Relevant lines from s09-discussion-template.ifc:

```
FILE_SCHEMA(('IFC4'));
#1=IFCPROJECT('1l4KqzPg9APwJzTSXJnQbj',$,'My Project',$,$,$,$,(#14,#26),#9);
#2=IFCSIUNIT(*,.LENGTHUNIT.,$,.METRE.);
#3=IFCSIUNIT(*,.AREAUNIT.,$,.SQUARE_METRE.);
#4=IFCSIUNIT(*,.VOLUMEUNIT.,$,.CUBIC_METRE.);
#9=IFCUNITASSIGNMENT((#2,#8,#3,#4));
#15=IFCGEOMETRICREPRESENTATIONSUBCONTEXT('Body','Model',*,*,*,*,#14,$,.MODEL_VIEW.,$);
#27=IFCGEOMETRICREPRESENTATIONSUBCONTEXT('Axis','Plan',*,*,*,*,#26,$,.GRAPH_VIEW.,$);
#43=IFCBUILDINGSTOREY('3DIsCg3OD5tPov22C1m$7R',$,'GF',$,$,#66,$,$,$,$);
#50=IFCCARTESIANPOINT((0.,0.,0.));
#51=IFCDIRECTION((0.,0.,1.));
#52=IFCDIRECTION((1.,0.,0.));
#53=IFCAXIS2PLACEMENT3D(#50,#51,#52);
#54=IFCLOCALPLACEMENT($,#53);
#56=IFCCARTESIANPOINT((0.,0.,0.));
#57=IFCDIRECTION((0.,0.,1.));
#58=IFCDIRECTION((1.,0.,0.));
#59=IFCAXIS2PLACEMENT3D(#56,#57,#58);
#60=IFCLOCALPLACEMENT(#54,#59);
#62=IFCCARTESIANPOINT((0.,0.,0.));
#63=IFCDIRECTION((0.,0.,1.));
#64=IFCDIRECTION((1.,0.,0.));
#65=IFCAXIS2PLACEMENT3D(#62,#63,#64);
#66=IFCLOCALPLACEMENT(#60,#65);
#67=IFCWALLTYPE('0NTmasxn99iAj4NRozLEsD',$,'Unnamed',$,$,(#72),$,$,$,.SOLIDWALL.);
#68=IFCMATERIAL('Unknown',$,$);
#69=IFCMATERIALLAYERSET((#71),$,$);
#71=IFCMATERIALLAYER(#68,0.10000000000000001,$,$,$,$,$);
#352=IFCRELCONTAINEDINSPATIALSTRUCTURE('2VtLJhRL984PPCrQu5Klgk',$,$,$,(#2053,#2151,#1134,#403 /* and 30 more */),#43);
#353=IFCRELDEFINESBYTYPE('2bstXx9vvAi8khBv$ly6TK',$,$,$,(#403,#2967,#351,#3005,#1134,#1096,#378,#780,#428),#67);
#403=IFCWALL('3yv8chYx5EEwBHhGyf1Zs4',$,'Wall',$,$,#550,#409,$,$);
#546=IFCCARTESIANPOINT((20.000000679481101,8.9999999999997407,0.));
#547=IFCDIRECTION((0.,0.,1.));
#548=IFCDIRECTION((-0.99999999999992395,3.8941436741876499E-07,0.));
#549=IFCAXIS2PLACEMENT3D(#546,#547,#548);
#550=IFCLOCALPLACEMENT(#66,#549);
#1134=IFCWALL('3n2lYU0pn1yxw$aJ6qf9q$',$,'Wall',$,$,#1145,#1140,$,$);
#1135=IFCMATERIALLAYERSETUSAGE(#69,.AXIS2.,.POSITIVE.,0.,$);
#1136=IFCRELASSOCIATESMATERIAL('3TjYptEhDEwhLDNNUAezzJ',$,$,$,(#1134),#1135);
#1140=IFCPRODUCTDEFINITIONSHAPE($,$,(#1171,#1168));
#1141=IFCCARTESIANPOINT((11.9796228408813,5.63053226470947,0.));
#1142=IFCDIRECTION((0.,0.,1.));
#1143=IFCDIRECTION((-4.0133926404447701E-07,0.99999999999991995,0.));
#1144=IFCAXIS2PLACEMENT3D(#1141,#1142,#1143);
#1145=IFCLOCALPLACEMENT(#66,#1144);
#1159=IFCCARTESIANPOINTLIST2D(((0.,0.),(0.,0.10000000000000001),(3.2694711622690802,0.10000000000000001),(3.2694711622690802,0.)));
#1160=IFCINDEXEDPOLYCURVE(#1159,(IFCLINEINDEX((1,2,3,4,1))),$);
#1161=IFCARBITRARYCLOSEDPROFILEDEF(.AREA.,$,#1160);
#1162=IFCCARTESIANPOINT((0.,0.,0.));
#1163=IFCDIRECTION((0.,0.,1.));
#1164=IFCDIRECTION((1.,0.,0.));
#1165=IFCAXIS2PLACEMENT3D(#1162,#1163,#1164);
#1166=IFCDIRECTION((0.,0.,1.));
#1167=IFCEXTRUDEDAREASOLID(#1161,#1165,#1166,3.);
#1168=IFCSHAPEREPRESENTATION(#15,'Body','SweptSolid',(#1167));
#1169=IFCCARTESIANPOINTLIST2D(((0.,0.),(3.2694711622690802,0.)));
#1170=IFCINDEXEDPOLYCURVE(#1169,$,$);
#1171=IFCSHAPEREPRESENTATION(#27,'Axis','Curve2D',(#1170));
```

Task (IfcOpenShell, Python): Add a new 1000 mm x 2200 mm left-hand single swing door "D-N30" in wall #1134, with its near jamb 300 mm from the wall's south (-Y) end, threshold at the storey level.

```python
import numpy as np
import ifcopenshell
import ifcopenshell.api.feature
import ifcopenshell.api.geometry
import ifcopenshell.api.root
import ifcopenshell.api.spatial
import ifcopenshell.geom
import ifcopenshell.util.element
import ifcopenshell.util.placement
import ifcopenshell.util.representation
import ifcopenshell.util.shape
import ifcopenshell.util.unit

model = ifcopenshell.open("s09-discussion-template.ifc")
unit_scale = ifcopenshell.util.unit.calculate_unit_scale(model)
settings = ifcopenshell.geom.settings()


def volume(element):
    """Net volume in cubic metres, openings subtracted."""
    shape = ifcopenshell.geom.create_shape(settings, element)
    return ifcopenshell.util.shape.get_volume(shape.geometry)


wall = model.by_guid("3n2lYU0pn1yxw$aJ6qf9q$")
storey = ifcopenshell.util.element.get_container(wall, ifc_class="IfcBuildingStorey")
context = ifcopenshell.util.representation.get_context(model, "Model", "Body", "MODEL_VIEW")
before = volume(wall)

width, height, from_end, sill = 1, 2.2, 0.3, 0.0  # metres

# The wall runs along its own X axis, and the end named is its -X end.
wall_shape = ifcopenshell.geom.create_shape(settings, wall)
x, y, z = ifcopenshell.util.shape.get_vertices(wall_shape.geometry).T
start = x.min() + from_end
face, thickness = float(y.min()), float(y.max() - y.min())
wall_matrix = ifcopenshell.util.placement.get_local_placement(wall.ObjectPlacement)
level = ifcopenshell.util.placement.get_local_placement(storey.ObjectPlacement)[2, 3]


def in_wall(x, y):
    """Placement at x, y metres in the wall's axes, at sill height."""
    matrix = wall_matrix.copy()
    matrix[:, 3] = wall_matrix @ np.array([x / unit_scale, y / unit_scale, 0.0, 1.0])
    matrix[2, 3] = level + sill / unit_scale
    return matrix


# Opening: a box that overshoots both wall faces by 50 mm.
opening = ifcopenshell.api.root.create_entity(model, ifc_class="IfcOpeningElement", predefined_type="OPENING")
box = ifcopenshell.api.geometry.add_wall_representation(
    model, context=context, length=width, height=height, thickness=thickness + 0.1
)
ifcopenshell.api.geometry.assign_representation(model, product=opening, representation=box)
ifcopenshell.api.geometry.edit_object_placement(model, product=opening, matrix=in_wall(start, face - 0.05), is_si=False)
ifcopenshell.api.feature.add_feature(model, feature=opening, element=wall)

door = ifcopenshell.api.root.create_entity(model, ifc_class="IfcDoor", name="D-N30", predefined_type="DOOR")
door.OverallWidth, door.OverallHeight = width / unit_scale, height / unit_scale
door.OperationType = "SINGLE_SWING_LEFT"
body = ifcopenshell.api.geometry.add_door_representation(
    model,
    context=context,
    overall_width=door.OverallWidth,
    overall_height=door.OverallHeight,
    operation_type="SINGLE_SWING_LEFT",
    lining_properties={"LiningDepth": thickness / unit_scale, "ThresholdDepth": thickness / unit_scale},
)
ifcopenshell.api.geometry.assign_representation(model, product=door, representation=body)
ifcopenshell.api.spatial.assign_container(model, products=[door], relating_structure=storey)
ifcopenshell.api.feature.add_filling(model, opening=opening, element=door)

# The lining spans the wall, so the door starts at the wall face.
ifcopenshell.api.geometry.edit_object_placement(model, product=door, matrix=in_wall(start, face), is_si=False)

after = volume(wall)

print(f"wall volume {before:.3f} -> {after:.3f} m3")

model.write("s09-discussion-template_v2.ifc")
```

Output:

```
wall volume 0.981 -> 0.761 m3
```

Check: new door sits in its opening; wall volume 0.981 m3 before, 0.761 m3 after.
